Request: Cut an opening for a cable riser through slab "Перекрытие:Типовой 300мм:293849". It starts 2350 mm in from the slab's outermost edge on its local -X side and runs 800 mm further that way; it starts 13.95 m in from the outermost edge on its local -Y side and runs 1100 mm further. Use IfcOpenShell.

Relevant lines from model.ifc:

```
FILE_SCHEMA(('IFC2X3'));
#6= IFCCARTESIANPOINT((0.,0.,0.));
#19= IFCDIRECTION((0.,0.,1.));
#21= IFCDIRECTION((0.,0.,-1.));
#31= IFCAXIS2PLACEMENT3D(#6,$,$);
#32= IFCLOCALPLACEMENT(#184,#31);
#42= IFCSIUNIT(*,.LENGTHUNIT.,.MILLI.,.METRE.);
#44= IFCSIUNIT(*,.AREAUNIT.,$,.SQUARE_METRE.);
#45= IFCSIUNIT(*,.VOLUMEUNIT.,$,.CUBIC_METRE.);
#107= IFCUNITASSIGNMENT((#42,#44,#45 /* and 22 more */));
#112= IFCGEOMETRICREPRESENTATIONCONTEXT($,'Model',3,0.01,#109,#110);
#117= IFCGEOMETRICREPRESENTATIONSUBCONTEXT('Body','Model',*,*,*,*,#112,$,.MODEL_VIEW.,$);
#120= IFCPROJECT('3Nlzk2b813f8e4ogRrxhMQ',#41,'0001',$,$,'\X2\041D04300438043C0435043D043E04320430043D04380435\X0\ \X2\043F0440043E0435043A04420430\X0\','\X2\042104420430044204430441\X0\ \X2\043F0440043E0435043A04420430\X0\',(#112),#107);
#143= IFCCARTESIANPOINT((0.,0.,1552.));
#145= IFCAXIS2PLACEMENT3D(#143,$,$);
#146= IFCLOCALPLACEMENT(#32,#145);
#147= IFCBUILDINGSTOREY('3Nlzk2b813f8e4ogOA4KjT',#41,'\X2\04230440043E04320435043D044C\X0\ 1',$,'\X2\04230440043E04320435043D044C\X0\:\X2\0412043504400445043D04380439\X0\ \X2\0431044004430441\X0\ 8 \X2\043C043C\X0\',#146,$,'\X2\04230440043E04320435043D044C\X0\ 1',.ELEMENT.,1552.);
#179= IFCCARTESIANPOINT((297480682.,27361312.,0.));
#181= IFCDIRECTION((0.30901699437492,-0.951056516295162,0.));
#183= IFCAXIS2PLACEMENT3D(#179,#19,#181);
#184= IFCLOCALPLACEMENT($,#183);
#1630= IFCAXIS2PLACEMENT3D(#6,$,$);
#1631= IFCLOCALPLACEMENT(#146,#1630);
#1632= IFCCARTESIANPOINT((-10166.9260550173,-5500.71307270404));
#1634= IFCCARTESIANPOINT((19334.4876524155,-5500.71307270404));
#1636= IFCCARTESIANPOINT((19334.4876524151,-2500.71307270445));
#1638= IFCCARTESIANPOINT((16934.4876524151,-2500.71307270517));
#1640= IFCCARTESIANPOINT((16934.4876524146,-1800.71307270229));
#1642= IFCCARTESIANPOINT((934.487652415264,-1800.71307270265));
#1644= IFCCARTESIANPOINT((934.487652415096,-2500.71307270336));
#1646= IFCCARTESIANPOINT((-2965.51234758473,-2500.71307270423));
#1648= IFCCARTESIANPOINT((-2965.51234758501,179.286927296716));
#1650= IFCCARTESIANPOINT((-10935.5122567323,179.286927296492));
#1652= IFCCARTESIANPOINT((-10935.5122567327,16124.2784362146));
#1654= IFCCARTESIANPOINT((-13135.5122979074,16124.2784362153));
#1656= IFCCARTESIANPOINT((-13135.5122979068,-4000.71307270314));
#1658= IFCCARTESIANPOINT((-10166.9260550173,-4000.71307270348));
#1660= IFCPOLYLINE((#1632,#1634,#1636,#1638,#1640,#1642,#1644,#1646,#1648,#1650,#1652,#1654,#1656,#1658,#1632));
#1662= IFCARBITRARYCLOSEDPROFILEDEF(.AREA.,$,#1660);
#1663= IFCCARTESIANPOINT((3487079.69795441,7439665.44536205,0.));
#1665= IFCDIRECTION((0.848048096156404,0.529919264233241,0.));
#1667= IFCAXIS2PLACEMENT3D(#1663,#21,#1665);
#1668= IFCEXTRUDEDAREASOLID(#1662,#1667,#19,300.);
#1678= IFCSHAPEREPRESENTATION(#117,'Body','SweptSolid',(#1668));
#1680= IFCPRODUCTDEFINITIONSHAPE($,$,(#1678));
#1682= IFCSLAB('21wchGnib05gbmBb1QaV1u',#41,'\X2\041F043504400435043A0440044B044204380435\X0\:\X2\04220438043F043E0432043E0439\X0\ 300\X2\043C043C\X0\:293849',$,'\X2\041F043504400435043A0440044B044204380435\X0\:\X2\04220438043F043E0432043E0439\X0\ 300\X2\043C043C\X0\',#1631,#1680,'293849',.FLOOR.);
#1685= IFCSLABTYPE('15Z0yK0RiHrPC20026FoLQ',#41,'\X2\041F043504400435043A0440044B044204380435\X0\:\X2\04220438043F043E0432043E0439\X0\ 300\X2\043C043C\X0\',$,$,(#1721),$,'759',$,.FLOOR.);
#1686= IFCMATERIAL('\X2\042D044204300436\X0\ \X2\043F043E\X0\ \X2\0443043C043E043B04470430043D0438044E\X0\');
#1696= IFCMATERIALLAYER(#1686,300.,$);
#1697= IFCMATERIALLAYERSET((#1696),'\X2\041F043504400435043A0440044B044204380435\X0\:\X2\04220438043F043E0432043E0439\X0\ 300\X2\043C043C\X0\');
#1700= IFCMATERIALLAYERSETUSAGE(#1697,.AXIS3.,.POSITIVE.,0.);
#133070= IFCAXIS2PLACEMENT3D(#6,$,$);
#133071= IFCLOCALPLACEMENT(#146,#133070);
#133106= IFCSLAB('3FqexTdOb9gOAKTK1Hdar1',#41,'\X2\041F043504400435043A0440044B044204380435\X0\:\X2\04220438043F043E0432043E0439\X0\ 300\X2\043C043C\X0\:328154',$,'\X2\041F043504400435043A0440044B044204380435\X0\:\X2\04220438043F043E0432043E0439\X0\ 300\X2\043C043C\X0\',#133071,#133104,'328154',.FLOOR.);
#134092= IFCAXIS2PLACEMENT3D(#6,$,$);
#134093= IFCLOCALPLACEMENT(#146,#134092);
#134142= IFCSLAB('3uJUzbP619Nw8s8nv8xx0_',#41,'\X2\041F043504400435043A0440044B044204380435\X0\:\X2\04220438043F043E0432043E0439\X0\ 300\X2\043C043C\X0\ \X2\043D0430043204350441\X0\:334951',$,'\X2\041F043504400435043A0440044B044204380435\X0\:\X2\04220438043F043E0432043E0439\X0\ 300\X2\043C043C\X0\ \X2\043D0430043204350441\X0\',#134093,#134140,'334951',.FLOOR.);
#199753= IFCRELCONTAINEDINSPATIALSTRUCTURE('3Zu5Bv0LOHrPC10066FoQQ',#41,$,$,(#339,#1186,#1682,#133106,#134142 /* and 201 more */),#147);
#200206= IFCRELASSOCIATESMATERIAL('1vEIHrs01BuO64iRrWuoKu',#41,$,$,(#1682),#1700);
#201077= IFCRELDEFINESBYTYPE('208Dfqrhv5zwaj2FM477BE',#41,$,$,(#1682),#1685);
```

```python
import numpy as np
import ifcopenshell
import ifcopenshell.api.feature
import ifcopenshell.api.geometry
import ifcopenshell.api.root
import ifcopenshell.geom
import ifcopenshell.util.placement
import ifcopenshell.util.representation
import ifcopenshell.util.shape
import ifcopenshell.util.unit

model = ifcopenshell.open("model.ifc")
unit_scale = ifcopenshell.util.unit.calculate_unit_scale(model)
settings = ifcopenshell.geom.settings()


def volume(element):
    """Net volume in cubic metres, openings subtracted."""
    shape = ifcopenshell.geom.create_shape(settings, element)
    return ifcopenshell.util.shape.get_volume(shape.geometry)


slab = model.by_guid("21wchGnib05gbmBb1QaV1u")
before = volume(slab)

# Extent in the slab's own axes, in metres. The edges named are its -X and -Y sides.
slab_shape = ifcopenshell.geom.create_shape(settings, slab)
vertices = ifcopenshell.util.shape.get_vertices(slab_shape.geometry)
x_min, y_min, bottom = vertices.min(axis=0)
top = vertices[:, 2].max()

opening = ifcopenshell.api.root.create_entity(model, ifc_class="IfcOpeningElement", name="Cable riser opening")
context = ifcopenshell.util.representation.get_context(model, "Model", "Body", "MODEL_VIEW")
width, depth = 0.8, 1.1
outline = [(0.0, 0.0), (width, 0.0), (width, depth), (0.0, depth), (0.0, 0.0)]
# Overshoot both faces by 50 mm so the cut is clean.
shape = ifcopenshell.api.geometry.add_slab_representation(
    model, context=context, depth=top - bottom + 0.1, polyline=outline
)
ifcopenshell.api.geometry.assign_representation(model, product=opening, representation=shape)

matrix = ifcopenshell.util.placement.get_local_placement(slab.ObjectPlacement)
matrix[:, 3] = matrix @ np.append(np.array([x_min + 2.35, y_min + 13.95, bottom - 0.05]) / unit_scale, 1.0)
ifcopenshell.api.geometry.edit_object_placement(model, product=opening, matrix=matrix, is_si=False)
ifcopenshell.api.feature.add_feature(model, feature=opening, element=slab)

after = volume(slab)

print(f"slab volume {before:.3f} -> {after:.3f} m3")

model.write("model_edited.ifc")
```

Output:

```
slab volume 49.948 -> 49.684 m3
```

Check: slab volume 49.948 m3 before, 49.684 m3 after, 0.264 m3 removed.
